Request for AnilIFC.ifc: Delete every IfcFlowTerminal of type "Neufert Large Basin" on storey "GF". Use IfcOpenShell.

First a look at what the model holds.

```python
import ifcopenshell
import ifcopenshell.util.element

model = ifcopenshell.open("AnilIFC.ifc")
print(model.schema)
storey = next(s for s in model.by_type("IfcBuildingStorey") if s.Name == "GF")
terminals = [e for e in ifcopenshell.util.element.get_decomposition(storey) if e.is_a("IfcFlowTerminal")]
seen = {}
for e in terminals:
    element_type = ifcopenshell.util.element.get_type(e)
    name = element_type.Name if element_type not in (None, e) else None
    seen[name] = seen.get(name, 0) + 1
for name, count in sorted(seen.items(), key=str):
    print(count, "x", name)
```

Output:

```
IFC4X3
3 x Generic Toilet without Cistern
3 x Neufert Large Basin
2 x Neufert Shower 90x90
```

```python
import ifcopenshell
import ifcopenshell.api.root
import ifcopenshell.util.element

model = ifcopenshell.open("AnilIFC.ifc")

storey = next(s for s in model.by_type("IfcBuildingStorey") if s.Name == "GF")
terminals = [e for e in ifcopenshell.util.element.get_decomposition(storey) if e.is_a("IfcFlowTerminal")]
targets = [e for e in terminals if (t := ifcopenshell.util.element.get_type(e)) not in (None, e) and t.Name == "Neufert Large Basin"]

for e in targets:
    ifcopenshell.api.root.remove_product(model, product=e)
print(len(targets), "removed")

model.write("AnilIFC_edited.ifc")
```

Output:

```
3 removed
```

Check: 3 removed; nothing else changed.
